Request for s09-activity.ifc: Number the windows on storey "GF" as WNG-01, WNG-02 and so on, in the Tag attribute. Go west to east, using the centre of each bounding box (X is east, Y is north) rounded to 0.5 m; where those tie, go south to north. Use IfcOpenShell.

First a look at what the model holds.

```python
import ifcopenshell
import ifcopenshell.util.element
import ifcopenshell.util.placement

model = ifcopenshell.open("s09-activity.ifc")
print(model.schema)
storey = next(s for s in model.by_type("IfcBuildingStorey") if s.Name == "GF")
windows = [e for e in ifcopenshell.util.element.get_decomposition(storey) if e.is_a("IfcWindow")]
for e in sorted(windows, key=lambda e: e.id()):
    origin = ifcopenshell.util.placement.get_local_placement(e.ObjectPlacement)[:3, 3]
    print(e.id(), e.Tag, e.Name, origin.round(2) + 0.0, sep=" | ")
```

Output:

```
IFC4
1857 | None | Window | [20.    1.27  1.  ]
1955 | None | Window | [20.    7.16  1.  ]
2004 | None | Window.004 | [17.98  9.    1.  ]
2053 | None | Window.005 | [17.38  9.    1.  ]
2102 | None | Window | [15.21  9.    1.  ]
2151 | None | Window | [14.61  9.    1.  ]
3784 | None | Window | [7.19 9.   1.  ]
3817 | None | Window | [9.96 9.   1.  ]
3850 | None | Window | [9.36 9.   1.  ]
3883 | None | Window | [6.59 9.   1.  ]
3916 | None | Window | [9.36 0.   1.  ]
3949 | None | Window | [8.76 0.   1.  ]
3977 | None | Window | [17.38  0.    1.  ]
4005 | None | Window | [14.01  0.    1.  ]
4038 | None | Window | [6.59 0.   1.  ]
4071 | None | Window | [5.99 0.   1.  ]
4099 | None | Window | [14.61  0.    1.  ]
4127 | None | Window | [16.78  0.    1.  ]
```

```python
import ifcopenshell
import ifcopenshell.geom
import ifcopenshell.util.element
import ifcopenshell.util.shape

model = ifcopenshell.open("s09-activity.ifc")
settings = ifcopenshell.geom.settings()
settings.set("use-world-coords", True)


def centre(element):
    shape = ifcopenshell.geom.create_shape(settings, element)
    return ifcopenshell.util.shape.get_bbox_centroid(shape.geometry)


storey = next(s for s in model.by_type("IfcBuildingStorey") if s.Name == "GF")
windows = [e for e in ifcopenshell.util.element.get_decomposition(storey) if e.is_a("IfcWindow")]

# Insertion points can sit at a corner or the storey origin, so sort by the geometry (in metres).
centres = {e: centre(e) for e in windows}
windows.sort(key=lambda e: (round(centres[e][0] / 0.5), centres[e][1]))

for i, e in enumerate(windows, start=1):
    number = f"WNG-{i:02d}"
    e.Tag = number
    print(e.id(), number)

model.write("s09-activity_updated.ifc")
```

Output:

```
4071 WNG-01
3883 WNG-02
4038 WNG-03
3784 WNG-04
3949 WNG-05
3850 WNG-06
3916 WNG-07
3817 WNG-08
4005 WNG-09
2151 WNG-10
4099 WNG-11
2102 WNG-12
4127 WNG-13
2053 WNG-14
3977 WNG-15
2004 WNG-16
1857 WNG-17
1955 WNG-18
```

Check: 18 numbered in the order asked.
